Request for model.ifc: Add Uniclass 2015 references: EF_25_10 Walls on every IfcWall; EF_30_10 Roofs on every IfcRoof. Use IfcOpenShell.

First a look at what the model holds.

```python
import ifcopenshell

model = ifcopenshell.open("model.ifc")
print(model.schema)
print("classifications:", [c.Name for c in model.by_type("IfcClassification")])
for ifc_class in ("IfcDoor", "IfcRoof", "IfcStair", "IfcWall", "IfcWindow"):
    print(ifc_class, len(model.by_type(ifc_class)))
```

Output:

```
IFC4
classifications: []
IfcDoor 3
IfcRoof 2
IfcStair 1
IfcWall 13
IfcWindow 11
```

```python
import ifcopenshell
import ifcopenshell.api.classification

model = ifcopenshell.open("model.ifc")

system = ifcopenshell.api.classification.add_classification(model, classification="Uniclass 2015")

codes = {
    "IfcWall": ("EF_25_10", "Walls"),
    "IfcRoof": ("EF_30_10", "Roofs"),
}
for ifc_class, (code, name) in codes.items():
    products = model.by_type(ifc_class)
    ifcopenshell.api.classification.add_reference(
        model, products=products, classification=system, identification=code, name=name
    )
    print(code, len(products))

model.write("model_updated.ifc")
```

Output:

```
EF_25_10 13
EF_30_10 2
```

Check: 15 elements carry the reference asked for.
